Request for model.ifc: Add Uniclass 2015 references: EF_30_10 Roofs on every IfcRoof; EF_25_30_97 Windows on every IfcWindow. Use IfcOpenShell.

First a look at what the model holds.

```python
import ifcopenshell

model = ifcopenshell.open("model.ifc")
print(model.schema)
print("classifications:", [c.Name for c in model.by_type("IfcClassification")])
for ifc_class in ("IfcDoor", "IfcRoof", "IfcStair", "IfcWall", "IfcWindow"):
    print(ifc_class, len(model.by_type(ifc_class)))
```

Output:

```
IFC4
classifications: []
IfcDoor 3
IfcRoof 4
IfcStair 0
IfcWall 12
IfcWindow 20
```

```python
import ifcopenshell
import ifcopenshell.api.classification

model = ifcopenshell.open("model.ifc")

system = ifcopenshell.api.classification.add_classification(model, classification="Uniclass 2015")

codes = {
    "IfcRoof": ("EF_30_10", "Roofs"),
    "IfcWindow": ("EF_25_30_97", "Windows"),
}
for ifc_class, (code, name) in codes.items():
    products = model.by_type(ifc_class)
    ifcopenshell.api.classification.add_reference(
        model, products=products, classification=system, identification=code, name=name
    )
    print(code, len(products))

model.write("model_updated.ifc")
```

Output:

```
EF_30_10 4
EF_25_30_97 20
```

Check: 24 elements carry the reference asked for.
